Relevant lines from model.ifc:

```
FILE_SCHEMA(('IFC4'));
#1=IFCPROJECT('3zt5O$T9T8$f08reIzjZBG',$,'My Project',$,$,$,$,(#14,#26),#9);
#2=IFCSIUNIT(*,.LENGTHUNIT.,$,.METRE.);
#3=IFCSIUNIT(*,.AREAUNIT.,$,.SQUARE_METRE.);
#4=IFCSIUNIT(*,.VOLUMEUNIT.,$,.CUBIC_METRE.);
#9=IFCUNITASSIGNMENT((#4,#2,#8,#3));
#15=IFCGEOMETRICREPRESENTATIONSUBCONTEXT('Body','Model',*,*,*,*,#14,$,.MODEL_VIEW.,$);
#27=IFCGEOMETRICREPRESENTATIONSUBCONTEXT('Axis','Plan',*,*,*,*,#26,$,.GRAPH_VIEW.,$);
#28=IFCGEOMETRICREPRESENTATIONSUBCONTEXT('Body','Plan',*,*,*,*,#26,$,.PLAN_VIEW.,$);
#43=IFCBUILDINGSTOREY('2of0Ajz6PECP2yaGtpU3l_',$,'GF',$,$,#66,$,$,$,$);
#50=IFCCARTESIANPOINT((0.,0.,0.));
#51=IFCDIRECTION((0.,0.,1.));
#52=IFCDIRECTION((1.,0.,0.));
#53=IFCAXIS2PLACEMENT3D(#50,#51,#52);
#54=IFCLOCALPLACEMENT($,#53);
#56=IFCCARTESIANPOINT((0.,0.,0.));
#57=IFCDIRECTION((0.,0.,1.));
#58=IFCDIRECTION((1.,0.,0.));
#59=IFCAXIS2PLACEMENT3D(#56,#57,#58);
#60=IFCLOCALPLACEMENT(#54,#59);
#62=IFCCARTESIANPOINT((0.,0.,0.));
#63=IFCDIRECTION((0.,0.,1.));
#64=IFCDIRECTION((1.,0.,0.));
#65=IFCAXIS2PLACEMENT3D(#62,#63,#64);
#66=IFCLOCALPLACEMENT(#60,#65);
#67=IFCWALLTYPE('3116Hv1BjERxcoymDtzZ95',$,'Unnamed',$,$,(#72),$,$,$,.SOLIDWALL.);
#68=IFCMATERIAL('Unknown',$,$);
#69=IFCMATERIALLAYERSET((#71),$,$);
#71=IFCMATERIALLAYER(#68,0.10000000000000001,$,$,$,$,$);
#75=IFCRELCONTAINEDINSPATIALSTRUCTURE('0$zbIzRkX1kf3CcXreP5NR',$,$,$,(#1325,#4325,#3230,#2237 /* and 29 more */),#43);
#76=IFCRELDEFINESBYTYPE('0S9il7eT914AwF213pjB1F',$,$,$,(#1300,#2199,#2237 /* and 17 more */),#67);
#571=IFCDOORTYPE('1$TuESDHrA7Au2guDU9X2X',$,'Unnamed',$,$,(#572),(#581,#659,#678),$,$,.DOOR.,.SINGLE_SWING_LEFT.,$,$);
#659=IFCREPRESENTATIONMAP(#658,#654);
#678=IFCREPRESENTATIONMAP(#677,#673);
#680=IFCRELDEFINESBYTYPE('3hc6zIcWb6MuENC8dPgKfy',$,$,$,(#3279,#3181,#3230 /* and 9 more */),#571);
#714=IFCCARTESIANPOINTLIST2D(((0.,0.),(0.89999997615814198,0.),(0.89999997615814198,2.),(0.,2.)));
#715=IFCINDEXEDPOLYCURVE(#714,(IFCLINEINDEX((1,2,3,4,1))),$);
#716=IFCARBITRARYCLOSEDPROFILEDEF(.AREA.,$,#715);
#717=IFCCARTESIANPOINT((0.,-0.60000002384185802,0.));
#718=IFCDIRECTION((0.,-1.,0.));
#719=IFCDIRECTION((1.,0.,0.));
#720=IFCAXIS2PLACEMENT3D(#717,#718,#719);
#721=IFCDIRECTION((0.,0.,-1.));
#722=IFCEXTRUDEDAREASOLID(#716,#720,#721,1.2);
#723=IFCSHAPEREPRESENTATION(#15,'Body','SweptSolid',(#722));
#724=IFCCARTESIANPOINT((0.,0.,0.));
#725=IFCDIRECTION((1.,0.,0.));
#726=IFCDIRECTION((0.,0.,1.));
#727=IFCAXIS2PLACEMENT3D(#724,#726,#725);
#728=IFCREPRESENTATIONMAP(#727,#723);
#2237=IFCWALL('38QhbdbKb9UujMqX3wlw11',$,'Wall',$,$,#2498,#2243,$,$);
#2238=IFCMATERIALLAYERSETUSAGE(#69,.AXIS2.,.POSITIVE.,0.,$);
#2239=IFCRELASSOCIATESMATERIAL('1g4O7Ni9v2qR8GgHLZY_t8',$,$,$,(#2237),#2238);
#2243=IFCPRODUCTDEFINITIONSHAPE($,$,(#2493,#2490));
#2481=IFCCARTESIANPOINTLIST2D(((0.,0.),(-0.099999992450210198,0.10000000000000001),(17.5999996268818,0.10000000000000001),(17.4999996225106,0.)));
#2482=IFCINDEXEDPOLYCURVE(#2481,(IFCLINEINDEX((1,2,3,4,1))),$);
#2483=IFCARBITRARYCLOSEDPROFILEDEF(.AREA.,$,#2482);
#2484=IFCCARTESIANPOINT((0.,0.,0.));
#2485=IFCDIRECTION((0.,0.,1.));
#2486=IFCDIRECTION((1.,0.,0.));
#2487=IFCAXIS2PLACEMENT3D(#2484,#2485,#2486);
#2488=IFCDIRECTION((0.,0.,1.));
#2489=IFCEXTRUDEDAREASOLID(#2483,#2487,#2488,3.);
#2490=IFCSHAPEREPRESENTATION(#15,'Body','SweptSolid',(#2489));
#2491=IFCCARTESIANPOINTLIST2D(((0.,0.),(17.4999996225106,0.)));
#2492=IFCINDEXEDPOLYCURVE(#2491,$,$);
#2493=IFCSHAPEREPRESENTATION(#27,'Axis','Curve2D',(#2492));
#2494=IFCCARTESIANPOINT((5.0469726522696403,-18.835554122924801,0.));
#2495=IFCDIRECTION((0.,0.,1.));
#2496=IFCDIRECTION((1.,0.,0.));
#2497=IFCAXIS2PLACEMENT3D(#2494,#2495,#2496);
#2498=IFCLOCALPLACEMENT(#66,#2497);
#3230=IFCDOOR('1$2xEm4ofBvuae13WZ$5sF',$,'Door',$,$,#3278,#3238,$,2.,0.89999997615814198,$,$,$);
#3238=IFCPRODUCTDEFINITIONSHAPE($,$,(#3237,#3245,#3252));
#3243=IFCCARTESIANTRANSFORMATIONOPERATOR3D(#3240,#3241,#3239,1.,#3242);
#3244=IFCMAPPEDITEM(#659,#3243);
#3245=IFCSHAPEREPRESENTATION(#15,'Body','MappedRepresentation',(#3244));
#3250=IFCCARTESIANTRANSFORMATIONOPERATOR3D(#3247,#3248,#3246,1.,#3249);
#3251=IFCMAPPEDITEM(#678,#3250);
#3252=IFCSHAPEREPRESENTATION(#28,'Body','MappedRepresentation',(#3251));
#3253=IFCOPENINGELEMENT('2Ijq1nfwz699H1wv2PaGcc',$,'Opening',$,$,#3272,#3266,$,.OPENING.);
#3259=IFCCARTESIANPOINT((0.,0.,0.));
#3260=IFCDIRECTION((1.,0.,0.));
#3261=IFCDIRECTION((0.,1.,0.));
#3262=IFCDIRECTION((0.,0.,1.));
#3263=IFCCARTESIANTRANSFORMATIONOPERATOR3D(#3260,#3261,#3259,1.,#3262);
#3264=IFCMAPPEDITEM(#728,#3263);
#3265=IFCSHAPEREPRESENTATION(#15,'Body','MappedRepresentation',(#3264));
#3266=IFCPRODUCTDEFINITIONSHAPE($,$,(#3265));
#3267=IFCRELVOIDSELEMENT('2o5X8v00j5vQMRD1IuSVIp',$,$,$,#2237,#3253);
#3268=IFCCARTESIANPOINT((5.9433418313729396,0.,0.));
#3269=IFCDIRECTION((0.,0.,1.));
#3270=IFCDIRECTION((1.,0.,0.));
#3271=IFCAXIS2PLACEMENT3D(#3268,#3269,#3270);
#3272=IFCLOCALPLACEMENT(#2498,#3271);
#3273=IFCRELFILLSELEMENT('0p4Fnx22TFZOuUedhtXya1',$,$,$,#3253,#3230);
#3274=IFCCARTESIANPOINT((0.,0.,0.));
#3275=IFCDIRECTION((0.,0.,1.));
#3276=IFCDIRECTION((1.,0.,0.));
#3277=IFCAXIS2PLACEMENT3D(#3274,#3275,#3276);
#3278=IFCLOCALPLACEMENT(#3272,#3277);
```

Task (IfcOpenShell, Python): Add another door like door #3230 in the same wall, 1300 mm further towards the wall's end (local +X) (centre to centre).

```python
import ifcopenshell
import ifcopenshell.api.feature
import ifcopenshell.api.geometry
import ifcopenshell.api.root
import ifcopenshell.geom
import ifcopenshell.util.element
import ifcopenshell.util.placement
import ifcopenshell.util.shape

model = ifcopenshell.open("model.ifc")
settings = ifcopenshell.geom.settings()


def volume(element):
    """Net volume in cubic metres, openings subtracted."""
    shape = ifcopenshell.geom.create_shape(settings, element)
    return ifcopenshell.util.shape.get_volume(shape.geometry)


door = model.by_id(3230)
opening = door.FillsVoids[0].RelatingOpeningElement
wall = opening.VoidsElements[0].RelatingBuildingElement
before = volume(wall)
shift = ifcopenshell.util.placement.get_local_placement(wall.ObjectPlacement)[:3, 0] * 1.3

# copy_class copies the void relationship, type, container and properties, but no geometry.
new_opening = ifcopenshell.api.root.copy_class(model, product=opening)
new_opening.Representation = ifcopenshell.util.element.copy_deep(
    model, opening.Representation, exclude=["IfcGeometricRepresentationContext", "IfcRepresentationMap"]
)
new_door = ifcopenshell.api.root.copy_class(model, product=door)
new_door.Representation = ifcopenshell.util.element.copy_deep(
    model, door.Representation, exclude=["IfcGeometricRepresentationContext", "IfcRepresentationMap"]
)
ifcopenshell.api.feature.add_filling(model, opening=new_opening, element=new_door)

for old, new in ((opening, new_opening), (door, new_door)):
    matrix = ifcopenshell.util.placement.get_local_placement(old.ObjectPlacement)
    matrix[:3, 3] += shift
    ifcopenshell.api.geometry.edit_object_placement(model, product=new, matrix=matrix, is_si=False)

after = volume(wall)

print(f"wall volume {before:.3f} -> {after:.3f} m3")

model.write("model-out.ifc")
```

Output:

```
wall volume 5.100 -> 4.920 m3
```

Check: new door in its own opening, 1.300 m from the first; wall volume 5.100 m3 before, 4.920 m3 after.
